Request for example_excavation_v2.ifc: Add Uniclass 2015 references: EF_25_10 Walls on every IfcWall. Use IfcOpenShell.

First a look at what the model holds.

```python
import ifcopenshell

model = ifcopenshell.open("example_excavation_v2.ifc")
print(model.schema)
print("classifications:", [c.Name for c in model.by_type("IfcClassification")])
for ifc_class in ("IfcDoor", "IfcRoof", "IfcStair", "IfcWall", "IfcWindow"):
    print(ifc_class, len(model.by_type(ifc_class)))
```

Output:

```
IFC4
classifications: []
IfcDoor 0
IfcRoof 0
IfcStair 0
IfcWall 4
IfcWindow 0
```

```python
import ifcopenshell
import ifcopenshell.api.classification

model = ifcopenshell.open("example_excavation_v2.ifc")

system = ifcopenshell.api.classification.add_classification(model, classification="Uniclass 2015")

codes = {
    "IfcWall": ("EF_25_10", "Walls"),
}
for ifc_class, (code, name) in codes.items():
    products = model.by_type(ifc_class)
    ifcopenshell.api.classification.add_reference(
        model, products=products, classification=system, identification=code, name=name
    )
    print(code, len(products))

model.write("example_excavation_v2_rev.ifc")
```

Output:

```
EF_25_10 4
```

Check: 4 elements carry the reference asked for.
